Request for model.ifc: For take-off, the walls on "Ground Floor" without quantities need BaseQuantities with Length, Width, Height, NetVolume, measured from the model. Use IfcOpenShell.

First a look at what the model holds.

```python
import ifcopenshell
import ifcopenshell.util.element
import ifcopenshell.util.unit

model = ifcopenshell.open("model.ifc")
print(model.schema)
for unit_type in ("LENGTHUNIT", "AREAUNIT", "VOLUMEUNIT"):
    print(unit_type, ifcopenshell.util.unit.calculate_unit_scale(model, unit_type))
storey = next(s for s in model.by_type("IfcBuildingStorey") if s.Name == "Ground Floor")
walls = [e for e in ifcopenshell.util.element.get_decomposition(storey) if e.is_a("IfcWall")]
for e in sorted(walls, key=lambda e: e.id()):
    print(e.id(), e.is_a(), e.Name, list(ifcopenshell.util.element.get_psets(e, qtos_only=True)), sep=" | ")
```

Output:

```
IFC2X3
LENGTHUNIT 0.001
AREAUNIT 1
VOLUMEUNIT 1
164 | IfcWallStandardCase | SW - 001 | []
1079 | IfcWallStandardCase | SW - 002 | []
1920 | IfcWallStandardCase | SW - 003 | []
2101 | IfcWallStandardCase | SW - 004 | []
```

```python
import ifcopenshell
import ifcopenshell.api.pset
import ifcopenshell.geom
import ifcopenshell.util.element
import ifcopenshell.util.shape
import ifcopenshell.util.unit

model = ifcopenshell.open("model.ifc")
unit_scale = ifcopenshell.util.unit.calculate_unit_scale(model)
volume_scale = ifcopenshell.util.unit.calculate_unit_scale(model, "VOLUMEUNIT")
settings = ifcopenshell.geom.settings()

storey = next(s for s in model.by_type("IfcBuildingStorey") if s.Name == "Ground Floor")
walls = [e for e in ifcopenshell.util.element.get_decomposition(storey) if e.is_a("IfcWall")]

for e in sorted(walls, key=lambda e: e.id()):
    if ifcopenshell.util.element.get_psets(e, qtos_only=True, should_inherit=False):
        continue
    # Geometry comes back in metres, in the element's own axes.
    shape = ifcopenshell.geom.create_shape(settings, e)
    values = {
        "Length": ifcopenshell.util.shape.get_x(shape.geometry) / unit_scale,
        "Width": ifcopenshell.util.shape.get_y(shape.geometry) / unit_scale,
        "Height": ifcopenshell.util.shape.get_z(shape.geometry) / unit_scale,
        "NetVolume": ifcopenshell.util.shape.get_volume(shape.geometry) / volume_scale,
    }
    qto = ifcopenshell.api.pset.add_qto(model, product=e, name="BaseQuantities")
    ifcopenshell.api.pset.edit_qto(model, qto=qto, properties=values)
    print(e.id(), {k: round(v, 3) for k, v in values.items()})

model.write("model_rev.ifc")
```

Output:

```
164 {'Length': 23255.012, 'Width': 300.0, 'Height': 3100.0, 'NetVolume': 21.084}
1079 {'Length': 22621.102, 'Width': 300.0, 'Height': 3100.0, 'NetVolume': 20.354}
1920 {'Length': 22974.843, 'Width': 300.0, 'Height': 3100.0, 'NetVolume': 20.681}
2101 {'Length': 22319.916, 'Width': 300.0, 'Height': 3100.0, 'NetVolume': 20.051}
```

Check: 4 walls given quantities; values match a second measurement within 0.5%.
